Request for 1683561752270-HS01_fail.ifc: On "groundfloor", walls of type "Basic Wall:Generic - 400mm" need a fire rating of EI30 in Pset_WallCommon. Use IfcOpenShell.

First a look at what the model holds.

```python
import ifcopenshell
import ifcopenshell.util.element

model = ifcopenshell.open("1683561752270-HS01_fail.ifc")
print(model.schema)
storey = next(s for s in model.by_type("IfcBuildingStorey") if s.Name == "groundfloor")
walls = [e for e in ifcopenshell.util.element.get_decomposition(storey) if e.is_a("IfcWall")]
seen = {}
for e in walls:
    element_type = ifcopenshell.util.element.get_type(e)
    key = (element_type.Name if element_type != e and element_type else None, ifcopenshell.util.element.get_pset(e, "Pset_WallCommon", "FireRating"))
    seen[key] = seen.get(key, 0) + 1
for (name, value), count in sorted(seen.items(), key=str):
    print(count, "x", name, "|", value)
```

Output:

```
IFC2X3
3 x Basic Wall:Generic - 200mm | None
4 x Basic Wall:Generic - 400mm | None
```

```python
import ifcopenshell
import ifcopenshell.api.pset
import ifcopenshell.util.element

model = ifcopenshell.open("1683561752270-HS01_fail.ifc")

storey = next(s for s in model.by_type("IfcBuildingStorey") if s.Name == "groundfloor")
walls = [e for e in ifcopenshell.util.element.get_decomposition(storey) if e.is_a("IfcWall")]

count = 0
for e in walls:
    element_type = ifcopenshell.util.element.get_type(e)
    if element_type in (None, e) or element_type.Name != "Basic Wall:Generic - 400mm":
        continue
    # add_pset returns the element's existing set when there is one.
    pset = ifcopenshell.api.pset.add_pset(model, product=e, name="Pset_WallCommon")
    ifcopenshell.api.pset.edit_pset(model, pset=pset, properties={"FireRating": "EI30"})
    count += 1

print(count, "walls updated")

model.write("1683561752270-HS01_fail_edited.ifc")
```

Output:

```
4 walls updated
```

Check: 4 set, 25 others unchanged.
